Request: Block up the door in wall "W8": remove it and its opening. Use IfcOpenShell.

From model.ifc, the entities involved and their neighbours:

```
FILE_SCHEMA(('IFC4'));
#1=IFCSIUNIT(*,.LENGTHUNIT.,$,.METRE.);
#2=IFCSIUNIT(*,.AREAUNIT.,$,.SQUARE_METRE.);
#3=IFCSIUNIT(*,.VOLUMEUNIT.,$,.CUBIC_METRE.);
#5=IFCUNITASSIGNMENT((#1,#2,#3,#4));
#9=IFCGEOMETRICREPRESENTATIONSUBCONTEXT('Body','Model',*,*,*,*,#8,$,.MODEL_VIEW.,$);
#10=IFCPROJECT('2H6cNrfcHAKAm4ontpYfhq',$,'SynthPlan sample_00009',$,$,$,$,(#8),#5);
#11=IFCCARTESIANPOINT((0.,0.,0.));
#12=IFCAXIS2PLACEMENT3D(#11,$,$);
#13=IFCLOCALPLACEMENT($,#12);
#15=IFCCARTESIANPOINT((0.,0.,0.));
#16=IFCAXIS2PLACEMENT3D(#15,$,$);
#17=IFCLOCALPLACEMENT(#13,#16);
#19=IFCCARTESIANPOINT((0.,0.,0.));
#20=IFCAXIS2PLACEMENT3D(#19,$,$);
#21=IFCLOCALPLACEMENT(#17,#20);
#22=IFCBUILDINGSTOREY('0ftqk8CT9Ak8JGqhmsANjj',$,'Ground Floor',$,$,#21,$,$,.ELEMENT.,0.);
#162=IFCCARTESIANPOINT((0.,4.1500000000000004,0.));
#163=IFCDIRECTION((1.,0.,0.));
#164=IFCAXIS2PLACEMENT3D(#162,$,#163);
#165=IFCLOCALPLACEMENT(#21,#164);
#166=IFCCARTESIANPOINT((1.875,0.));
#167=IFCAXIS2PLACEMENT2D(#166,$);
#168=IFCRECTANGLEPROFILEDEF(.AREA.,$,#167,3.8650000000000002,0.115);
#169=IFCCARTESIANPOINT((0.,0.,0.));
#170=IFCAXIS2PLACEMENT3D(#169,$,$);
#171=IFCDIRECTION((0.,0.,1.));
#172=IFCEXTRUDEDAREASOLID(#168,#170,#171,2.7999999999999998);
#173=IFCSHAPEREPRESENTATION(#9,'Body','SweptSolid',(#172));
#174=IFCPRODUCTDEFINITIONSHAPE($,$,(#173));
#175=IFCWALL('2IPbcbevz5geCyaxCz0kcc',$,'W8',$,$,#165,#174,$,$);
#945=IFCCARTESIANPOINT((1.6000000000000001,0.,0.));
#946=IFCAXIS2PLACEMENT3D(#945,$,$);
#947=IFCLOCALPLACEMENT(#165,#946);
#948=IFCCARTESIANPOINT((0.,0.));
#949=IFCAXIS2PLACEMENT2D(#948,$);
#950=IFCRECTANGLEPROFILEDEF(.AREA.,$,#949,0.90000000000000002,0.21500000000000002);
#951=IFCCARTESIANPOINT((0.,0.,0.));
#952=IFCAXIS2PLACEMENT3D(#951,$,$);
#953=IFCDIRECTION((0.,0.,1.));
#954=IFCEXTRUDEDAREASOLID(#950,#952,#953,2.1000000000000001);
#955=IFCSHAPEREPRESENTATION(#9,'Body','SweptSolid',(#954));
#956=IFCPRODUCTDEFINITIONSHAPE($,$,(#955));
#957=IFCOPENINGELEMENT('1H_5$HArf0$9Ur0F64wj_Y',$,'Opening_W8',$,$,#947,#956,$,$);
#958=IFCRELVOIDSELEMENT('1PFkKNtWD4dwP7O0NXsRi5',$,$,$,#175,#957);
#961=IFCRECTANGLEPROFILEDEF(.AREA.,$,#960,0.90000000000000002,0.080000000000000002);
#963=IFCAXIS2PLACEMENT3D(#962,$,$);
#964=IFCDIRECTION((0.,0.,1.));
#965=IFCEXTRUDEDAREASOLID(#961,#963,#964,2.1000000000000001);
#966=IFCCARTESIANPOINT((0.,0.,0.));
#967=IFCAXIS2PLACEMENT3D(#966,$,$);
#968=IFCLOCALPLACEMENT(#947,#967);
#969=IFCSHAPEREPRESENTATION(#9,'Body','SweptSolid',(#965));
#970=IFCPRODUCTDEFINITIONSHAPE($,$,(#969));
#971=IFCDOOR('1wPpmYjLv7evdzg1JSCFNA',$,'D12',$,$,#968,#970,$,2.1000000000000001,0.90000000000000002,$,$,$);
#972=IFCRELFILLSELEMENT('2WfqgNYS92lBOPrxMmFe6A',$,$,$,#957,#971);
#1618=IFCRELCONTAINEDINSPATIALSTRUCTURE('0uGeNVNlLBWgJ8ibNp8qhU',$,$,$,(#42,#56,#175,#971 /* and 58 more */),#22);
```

```python
import ifcopenshell
import ifcopenshell.api.feature
import ifcopenshell.api.root
import ifcopenshell.geom
import ifcopenshell.util.shape

model = ifcopenshell.open("model.ifc")
settings = ifcopenshell.geom.settings()


def volume(element):
    """Net volume in cubic metres, openings subtracted."""
    shape = ifcopenshell.geom.create_shape(settings, element)
    return ifcopenshell.util.shape.get_volume(shape.geometry)


door = model.by_id(971)
opening = door.FillsVoids[0].RelatingOpeningElement
wall = opening.VoidsElements[0].RelatingBuildingElement
before = volume(wall)

ifcopenshell.api.root.remove_product(model, product=door)
ifcopenshell.api.feature.remove_feature(model, feature=opening)

after = volume(wall)

print(f"wall volume {before:.3f} -> {after:.3f} m3")

model.write("model_rev.ifc")
```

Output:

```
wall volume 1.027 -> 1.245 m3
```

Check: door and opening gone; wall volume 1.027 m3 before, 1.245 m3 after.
